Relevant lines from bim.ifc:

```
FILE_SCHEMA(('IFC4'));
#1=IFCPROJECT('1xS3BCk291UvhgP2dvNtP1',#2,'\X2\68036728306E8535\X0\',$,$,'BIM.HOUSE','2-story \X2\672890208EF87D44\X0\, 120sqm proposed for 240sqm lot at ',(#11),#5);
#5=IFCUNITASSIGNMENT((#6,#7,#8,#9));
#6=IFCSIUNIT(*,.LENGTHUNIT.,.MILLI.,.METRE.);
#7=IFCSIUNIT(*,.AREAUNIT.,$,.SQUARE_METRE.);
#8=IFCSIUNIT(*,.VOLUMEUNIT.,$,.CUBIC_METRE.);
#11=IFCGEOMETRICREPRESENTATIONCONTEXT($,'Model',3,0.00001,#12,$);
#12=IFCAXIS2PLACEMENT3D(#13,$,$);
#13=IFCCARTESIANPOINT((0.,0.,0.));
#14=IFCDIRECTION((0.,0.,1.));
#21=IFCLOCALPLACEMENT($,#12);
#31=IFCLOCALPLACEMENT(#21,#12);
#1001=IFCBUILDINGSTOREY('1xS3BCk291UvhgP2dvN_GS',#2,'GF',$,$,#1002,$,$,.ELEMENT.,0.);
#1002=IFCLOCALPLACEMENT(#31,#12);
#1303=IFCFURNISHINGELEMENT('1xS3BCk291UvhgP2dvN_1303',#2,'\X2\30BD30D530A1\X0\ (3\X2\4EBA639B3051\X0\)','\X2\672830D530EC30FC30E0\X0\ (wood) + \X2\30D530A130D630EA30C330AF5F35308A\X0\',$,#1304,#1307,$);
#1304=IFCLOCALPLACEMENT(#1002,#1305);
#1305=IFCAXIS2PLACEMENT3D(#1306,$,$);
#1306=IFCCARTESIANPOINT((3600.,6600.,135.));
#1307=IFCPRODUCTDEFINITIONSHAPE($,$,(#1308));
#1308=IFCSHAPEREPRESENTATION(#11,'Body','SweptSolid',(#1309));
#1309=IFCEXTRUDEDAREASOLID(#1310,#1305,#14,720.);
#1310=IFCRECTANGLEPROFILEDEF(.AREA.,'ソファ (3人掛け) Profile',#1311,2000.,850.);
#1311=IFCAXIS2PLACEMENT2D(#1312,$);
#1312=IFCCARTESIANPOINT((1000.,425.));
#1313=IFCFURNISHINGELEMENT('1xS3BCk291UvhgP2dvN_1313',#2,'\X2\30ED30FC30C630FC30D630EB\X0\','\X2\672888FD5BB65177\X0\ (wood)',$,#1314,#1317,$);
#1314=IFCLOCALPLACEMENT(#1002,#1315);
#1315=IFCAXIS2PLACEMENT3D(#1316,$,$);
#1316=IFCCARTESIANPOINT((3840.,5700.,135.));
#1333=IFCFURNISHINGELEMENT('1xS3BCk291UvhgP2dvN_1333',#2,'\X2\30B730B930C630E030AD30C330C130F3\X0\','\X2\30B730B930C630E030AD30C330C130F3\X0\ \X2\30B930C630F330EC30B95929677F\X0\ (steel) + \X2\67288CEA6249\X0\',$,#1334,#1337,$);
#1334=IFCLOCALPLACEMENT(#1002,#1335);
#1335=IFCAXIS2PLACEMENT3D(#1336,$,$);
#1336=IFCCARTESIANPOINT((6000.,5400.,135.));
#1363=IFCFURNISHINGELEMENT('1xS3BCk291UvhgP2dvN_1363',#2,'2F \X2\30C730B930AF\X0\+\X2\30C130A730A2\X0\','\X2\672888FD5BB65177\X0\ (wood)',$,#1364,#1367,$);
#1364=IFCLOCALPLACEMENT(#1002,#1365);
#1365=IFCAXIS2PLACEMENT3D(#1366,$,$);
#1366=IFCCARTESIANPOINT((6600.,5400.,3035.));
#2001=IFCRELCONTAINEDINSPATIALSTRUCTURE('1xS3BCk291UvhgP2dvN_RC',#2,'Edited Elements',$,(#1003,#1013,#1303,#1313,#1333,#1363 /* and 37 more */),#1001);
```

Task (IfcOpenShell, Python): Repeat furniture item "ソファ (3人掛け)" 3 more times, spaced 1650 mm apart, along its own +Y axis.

```python
import ifcopenshell
import ifcopenshell.api.geometry
import ifcopenshell.api.root
import ifcopenshell.util.element
import ifcopenshell.util.placement

model = ifcopenshell.open("bim.ifc")


def reuse_history(source, copy):
    """copy_class also copies each property set's owner history, people and application; keep the originals."""
    for rel in copy.IsDefinedBy:
        if rel.is_a("IfcRelDefinesByProperties") and (history := rel.RelatingPropertyDefinition.OwnerHistory):
            rel.RelatingPropertyDefinition.OwnerHistory = source.OwnerHistory
            ifcopenshell.util.element.remove_deep2(model, history)


source = model.by_guid("1xS3BCk291UvhgP2dvN_1303")
base = ifcopenshell.util.placement.get_local_placement(source.ObjectPlacement)
step = base[:3, 1] * 1650.0

for i in range(1, 4):
    copy = ifcopenshell.api.root.copy_class(model, product=source)
    copy.Representation = ifcopenshell.util.element.copy_deep(
        model, source.Representation, exclude=["IfcGeometricRepresentationContext", "IfcRepresentationMap"]
    )
    reuse_history(source, copy)
    matrix = base.copy()
    matrix[:3, 3] += i * step
    print("added at", matrix[:3, 3].round(3) + 0.0)
    ifcopenshell.api.geometry.edit_object_placement(model, product=copy, matrix=matrix, is_si=False)

model.write("bim_edited.ifc")
```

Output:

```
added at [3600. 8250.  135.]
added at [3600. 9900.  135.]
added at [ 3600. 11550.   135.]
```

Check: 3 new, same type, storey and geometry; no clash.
